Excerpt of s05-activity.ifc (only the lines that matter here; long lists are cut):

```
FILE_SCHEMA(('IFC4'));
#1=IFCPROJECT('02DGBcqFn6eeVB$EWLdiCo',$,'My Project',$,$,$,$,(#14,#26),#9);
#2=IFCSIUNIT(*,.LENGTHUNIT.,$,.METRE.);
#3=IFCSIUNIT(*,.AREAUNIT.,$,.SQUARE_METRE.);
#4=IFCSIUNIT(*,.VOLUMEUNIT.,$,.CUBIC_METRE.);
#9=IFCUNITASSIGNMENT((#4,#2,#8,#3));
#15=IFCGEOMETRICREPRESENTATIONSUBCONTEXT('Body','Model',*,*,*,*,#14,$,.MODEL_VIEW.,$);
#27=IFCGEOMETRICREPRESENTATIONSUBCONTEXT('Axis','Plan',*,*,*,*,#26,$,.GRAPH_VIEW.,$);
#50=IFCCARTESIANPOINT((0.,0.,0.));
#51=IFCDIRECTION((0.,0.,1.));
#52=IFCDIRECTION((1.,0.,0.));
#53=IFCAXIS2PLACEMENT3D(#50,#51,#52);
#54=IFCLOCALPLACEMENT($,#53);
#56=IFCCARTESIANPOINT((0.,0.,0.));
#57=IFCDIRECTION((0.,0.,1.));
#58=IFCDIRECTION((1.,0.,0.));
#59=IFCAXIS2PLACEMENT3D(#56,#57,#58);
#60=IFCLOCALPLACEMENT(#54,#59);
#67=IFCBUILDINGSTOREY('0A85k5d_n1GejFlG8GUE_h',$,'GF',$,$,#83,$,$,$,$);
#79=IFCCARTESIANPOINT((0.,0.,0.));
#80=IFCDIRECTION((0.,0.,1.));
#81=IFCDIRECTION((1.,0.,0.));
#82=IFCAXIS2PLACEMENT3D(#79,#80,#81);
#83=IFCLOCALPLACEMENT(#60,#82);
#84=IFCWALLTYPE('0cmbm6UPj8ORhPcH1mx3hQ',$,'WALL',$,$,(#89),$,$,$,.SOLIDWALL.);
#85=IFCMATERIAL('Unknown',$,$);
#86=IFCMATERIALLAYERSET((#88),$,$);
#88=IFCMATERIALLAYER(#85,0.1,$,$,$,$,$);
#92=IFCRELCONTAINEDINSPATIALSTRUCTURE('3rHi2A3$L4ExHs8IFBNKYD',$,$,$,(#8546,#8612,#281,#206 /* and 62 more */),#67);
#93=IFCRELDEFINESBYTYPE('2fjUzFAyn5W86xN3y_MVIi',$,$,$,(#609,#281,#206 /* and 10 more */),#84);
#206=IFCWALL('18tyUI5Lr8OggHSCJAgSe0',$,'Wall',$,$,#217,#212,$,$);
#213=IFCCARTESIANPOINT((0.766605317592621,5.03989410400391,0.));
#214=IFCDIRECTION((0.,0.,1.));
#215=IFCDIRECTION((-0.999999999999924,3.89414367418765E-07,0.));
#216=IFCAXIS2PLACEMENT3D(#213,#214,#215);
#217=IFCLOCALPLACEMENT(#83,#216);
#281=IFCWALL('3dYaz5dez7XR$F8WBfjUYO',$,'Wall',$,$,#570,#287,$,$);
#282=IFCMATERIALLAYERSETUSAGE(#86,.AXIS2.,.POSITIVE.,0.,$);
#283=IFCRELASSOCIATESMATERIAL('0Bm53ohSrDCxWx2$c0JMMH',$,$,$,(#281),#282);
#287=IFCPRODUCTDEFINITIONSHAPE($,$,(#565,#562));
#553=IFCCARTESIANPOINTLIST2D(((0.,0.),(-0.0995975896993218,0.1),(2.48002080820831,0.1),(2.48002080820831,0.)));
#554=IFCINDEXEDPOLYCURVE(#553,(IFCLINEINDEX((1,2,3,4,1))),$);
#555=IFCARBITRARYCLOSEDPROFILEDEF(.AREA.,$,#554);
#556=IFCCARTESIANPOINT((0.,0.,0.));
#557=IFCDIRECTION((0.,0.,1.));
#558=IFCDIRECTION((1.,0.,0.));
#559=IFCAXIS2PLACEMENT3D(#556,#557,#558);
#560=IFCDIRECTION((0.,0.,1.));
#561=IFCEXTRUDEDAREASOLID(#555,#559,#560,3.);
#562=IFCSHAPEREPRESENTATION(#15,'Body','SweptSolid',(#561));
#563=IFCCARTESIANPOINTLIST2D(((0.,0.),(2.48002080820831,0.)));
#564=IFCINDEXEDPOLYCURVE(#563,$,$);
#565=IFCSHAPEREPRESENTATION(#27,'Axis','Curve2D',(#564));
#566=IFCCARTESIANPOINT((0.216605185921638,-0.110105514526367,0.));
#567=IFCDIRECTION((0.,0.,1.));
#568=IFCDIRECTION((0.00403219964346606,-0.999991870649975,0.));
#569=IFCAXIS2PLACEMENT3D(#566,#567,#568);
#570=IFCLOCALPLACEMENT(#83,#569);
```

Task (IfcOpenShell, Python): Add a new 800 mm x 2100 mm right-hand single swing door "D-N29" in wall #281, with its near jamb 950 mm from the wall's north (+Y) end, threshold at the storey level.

```python
import numpy as np
import ifcopenshell
import ifcopenshell.api.feature
import ifcopenshell.api.geometry
import ifcopenshell.api.root
import ifcopenshell.api.spatial
import ifcopenshell.geom
import ifcopenshell.util.element
import ifcopenshell.util.placement
import ifcopenshell.util.representation
import ifcopenshell.util.shape
import ifcopenshell.util.unit

model = ifcopenshell.open("s05-activity.ifc")
unit_scale = ifcopenshell.util.unit.calculate_unit_scale(model)
settings = ifcopenshell.geom.settings()


def volume(element):
    """Net volume in cubic metres, openings subtracted."""
    shape = ifcopenshell.geom.create_shape(settings, element)
    return ifcopenshell.util.shape.get_volume(shape.geometry)


wall = model.by_guid("3dYaz5dez7XR$F8WBfjUYO")
storey = ifcopenshell.util.element.get_container(wall, ifc_class="IfcBuildingStorey")
context = ifcopenshell.util.representation.get_context(model, "Model", "Body", "MODEL_VIEW")
before = volume(wall)

width, height, from_end, sill = 0.8, 2.1, 0.95, 0.0  # metres

# The wall runs along its own X axis, and the end named is its -X end.
wall_shape = ifcopenshell.geom.create_shape(settings, wall)
x, y, z = ifcopenshell.util.shape.get_vertices(wall_shape.geometry).T
start = x.min() + from_end
face, thickness = float(y.min()), float(y.max() - y.min())
wall_matrix = ifcopenshell.util.placement.get_local_placement(wall.ObjectPlacement)
level = ifcopenshell.util.placement.get_local_placement(storey.ObjectPlacement)[2, 3]


def in_wall(x, y):
    """Placement at x, y metres in the wall's axes, at sill height."""
    matrix = wall_matrix.copy()
    matrix[:, 3] = wall_matrix @ np.array([x / unit_scale, y / unit_scale, 0.0, 1.0])
    matrix[2, 3] = level + sill / unit_scale
    return matrix


# Opening: a box that overshoots both wall faces by 50 mm.
opening = ifcopenshell.api.root.create_entity(model, ifc_class="IfcOpeningElement", predefined_type="OPENING")
box = ifcopenshell.api.geometry.add_wall_representation(
    model, context=context, length=width, height=height, thickness=thickness + 0.1
)
ifcopenshell.api.geometry.assign_representation(model, product=opening, representation=box)
ifcopenshell.api.geometry.edit_object_placement(model, product=opening, matrix=in_wall(start, face - 0.05), is_si=False)
ifcopenshell.api.feature.add_feature(model, feature=opening, element=wall)

door = ifcopenshell.api.root.create_entity(model, ifc_class="IfcDoor", name="D-N29", predefined_type="DOOR")
door.OverallWidth, door.OverallHeight = width / unit_scale, height / unit_scale
door.OperationType = "SINGLE_SWING_RIGHT"
body = ifcopenshell.api.geometry.add_door_representation(
    model,
    context=context,
    overall_width=door.OverallWidth,
    overall_height=door.OverallHeight,
    operation_type="SINGLE_SWING_RIGHT",
    lining_properties={"LiningDepth": thickness / unit_scale, "ThresholdDepth": thickness / unit_scale},
)
ifcopenshell.api.geometry.assign_representation(model, product=door, representation=body)
ifcopenshell.api.spatial.assign_container(model, products=[door], relating_structure=storey)
ifcopenshell.api.feature.add_filling(model, opening=opening, element=door)

# The lining spans the wall, so the door starts at the wall face.
ifcopenshell.api.geometry.edit_object_placement(model, product=door, matrix=in_wall(start, face), is_si=False)

after = volume(wall)

print(f"wall volume {before:.3f} -> {after:.3f} m3")

model.write("s05-activity-out.ifc")
```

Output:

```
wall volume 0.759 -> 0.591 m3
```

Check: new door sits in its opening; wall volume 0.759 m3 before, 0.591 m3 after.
